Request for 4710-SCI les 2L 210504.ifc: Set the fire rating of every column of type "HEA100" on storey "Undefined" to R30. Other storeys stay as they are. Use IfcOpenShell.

First a look at what the model holds.

```python
import ifcopenshell
import ifcopenshell.util.element

model = ifcopenshell.open("4710-SCI les 2L 210504.ifc")
print(model.schema)
storey = next(s for s in model.by_type("IfcBuildingStorey") if s.Name == "Undefined")
columns = [e for e in ifcopenshell.util.element.get_decomposition(storey) if e.is_a("IfcColumn")]
seen = {}
for e in columns:
    element_type = ifcopenshell.util.element.get_type(e)
    key = (element_type.Name if element_type != e and element_type else None, ifcopenshell.util.element.get_pset(e, "Pset_ColumnCommon", "FireRating"))
    seen[key] = seen.get(key, 0) + 1
for (name, value), count in sorted(seen.items(), key=str):
    print(count, "x", name, "|", value)
```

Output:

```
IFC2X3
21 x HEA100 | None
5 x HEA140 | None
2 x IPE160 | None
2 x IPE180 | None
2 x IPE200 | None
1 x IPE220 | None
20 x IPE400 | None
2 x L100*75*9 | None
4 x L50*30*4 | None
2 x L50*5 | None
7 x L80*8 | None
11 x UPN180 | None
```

```python
import ifcopenshell
import ifcopenshell.api.pset
import ifcopenshell.util.element

model = ifcopenshell.open("4710-SCI les 2L 210504.ifc")

storey = next(s for s in model.by_type("IfcBuildingStorey") if s.Name == "Undefined")
columns = [e for e in ifcopenshell.util.element.get_decomposition(storey) if e.is_a("IfcColumn")]

count = 0
for e in columns:
    element_type = ifcopenshell.util.element.get_type(e)
    if element_type in (None, e) or element_type.Name != "HEA100":
        continue
    found = ifcopenshell.util.element.get_pset(e, "Pset_ColumnCommon", should_inherit=False)
    if found:
        pset = model.by_id(found["id"])
        if len(ifcopenshell.util.element.get_elements_by_pset(pset)) > 1:
            pset = ifcopenshell.api.pset.unshare_pset(model, products=[e], pset=pset)[0]
    else:
        pset = ifcopenshell.api.pset.add_pset(model, product=e, name="Pset_ColumnCommon")
    ifcopenshell.api.pset.edit_pset(model, pset=pset, properties={"FireRating": "R30"})
    count += 1

print(count, "columns updated")

model.write("4710-SCI les 2L 210504_updated.ifc")
```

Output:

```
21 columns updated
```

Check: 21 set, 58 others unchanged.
